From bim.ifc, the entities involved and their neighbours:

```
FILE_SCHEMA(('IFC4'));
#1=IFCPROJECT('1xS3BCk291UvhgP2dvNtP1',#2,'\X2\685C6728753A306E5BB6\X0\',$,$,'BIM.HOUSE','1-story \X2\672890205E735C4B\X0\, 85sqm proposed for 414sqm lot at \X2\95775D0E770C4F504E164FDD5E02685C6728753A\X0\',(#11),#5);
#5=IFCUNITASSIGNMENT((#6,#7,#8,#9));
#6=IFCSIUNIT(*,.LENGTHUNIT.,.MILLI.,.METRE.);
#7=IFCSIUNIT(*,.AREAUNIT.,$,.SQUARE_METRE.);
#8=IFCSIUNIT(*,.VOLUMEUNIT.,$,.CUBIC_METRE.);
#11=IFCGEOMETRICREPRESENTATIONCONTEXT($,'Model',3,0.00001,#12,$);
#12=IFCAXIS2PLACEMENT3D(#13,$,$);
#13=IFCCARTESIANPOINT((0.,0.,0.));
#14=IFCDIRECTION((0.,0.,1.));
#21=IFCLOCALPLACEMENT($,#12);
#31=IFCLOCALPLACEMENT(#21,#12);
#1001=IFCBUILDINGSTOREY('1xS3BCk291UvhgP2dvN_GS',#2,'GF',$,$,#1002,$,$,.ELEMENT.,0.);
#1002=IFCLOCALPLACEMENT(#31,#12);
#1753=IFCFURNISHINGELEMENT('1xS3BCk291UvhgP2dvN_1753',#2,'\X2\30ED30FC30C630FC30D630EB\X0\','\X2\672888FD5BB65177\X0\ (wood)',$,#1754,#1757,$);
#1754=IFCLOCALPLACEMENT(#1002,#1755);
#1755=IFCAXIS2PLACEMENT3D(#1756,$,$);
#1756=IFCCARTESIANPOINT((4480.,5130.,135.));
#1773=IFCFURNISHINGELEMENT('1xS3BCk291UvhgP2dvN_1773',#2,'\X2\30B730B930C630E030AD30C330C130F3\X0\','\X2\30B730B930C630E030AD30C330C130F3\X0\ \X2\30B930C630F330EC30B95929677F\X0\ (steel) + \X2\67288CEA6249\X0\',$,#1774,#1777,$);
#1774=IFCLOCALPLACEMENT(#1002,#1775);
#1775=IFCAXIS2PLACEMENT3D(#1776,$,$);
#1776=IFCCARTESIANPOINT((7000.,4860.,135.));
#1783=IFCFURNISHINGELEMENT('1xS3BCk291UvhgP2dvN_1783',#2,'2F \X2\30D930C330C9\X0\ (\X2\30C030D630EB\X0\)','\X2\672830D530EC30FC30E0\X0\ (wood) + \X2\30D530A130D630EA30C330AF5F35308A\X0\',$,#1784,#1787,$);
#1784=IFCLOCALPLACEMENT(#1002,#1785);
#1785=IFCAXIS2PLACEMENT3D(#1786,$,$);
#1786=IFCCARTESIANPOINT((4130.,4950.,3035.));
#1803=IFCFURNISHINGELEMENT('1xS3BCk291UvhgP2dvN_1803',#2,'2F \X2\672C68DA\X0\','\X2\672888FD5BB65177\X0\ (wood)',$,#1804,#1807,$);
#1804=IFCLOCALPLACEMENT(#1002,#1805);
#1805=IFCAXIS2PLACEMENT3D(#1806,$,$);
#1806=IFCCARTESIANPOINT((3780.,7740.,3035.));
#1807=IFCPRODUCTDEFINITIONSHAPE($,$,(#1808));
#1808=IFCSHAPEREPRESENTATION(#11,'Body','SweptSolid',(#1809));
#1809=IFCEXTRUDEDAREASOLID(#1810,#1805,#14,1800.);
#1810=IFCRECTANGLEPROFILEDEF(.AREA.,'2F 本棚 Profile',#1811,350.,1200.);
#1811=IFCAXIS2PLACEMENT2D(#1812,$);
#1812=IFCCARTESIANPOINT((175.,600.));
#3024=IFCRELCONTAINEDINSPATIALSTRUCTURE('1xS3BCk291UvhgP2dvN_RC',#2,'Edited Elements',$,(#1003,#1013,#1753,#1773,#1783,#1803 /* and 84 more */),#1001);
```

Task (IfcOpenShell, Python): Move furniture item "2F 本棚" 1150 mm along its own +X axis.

```python
import ifcopenshell
import ifcopenshell.api.geometry
import ifcopenshell.util.placement
import ifcopenshell.util.unit

model = ifcopenshell.open("bim.ifc")
unit_scale = ifcopenshell.util.unit.calculate_unit_scale(model)

item = model.by_guid("1xS3BCk291UvhgP2dvN_1803")
matrix = ifcopenshell.util.placement.get_local_placement(item.ObjectPlacement)
matrix[:3, 3] += matrix[:3, 0] * 1.15 / unit_scale
ifcopenshell.api.geometry.edit_object_placement(model, product=item, matrix=matrix, is_si=False)

print(ifcopenshell.util.placement.get_local_placement(item.ObjectPlacement).round(3) + 0.0)

model.write("bim_edited.ifc")
```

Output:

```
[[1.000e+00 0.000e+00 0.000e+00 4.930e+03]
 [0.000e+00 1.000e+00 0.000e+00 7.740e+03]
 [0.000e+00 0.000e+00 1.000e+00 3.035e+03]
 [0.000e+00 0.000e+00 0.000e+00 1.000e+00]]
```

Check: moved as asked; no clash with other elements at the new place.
